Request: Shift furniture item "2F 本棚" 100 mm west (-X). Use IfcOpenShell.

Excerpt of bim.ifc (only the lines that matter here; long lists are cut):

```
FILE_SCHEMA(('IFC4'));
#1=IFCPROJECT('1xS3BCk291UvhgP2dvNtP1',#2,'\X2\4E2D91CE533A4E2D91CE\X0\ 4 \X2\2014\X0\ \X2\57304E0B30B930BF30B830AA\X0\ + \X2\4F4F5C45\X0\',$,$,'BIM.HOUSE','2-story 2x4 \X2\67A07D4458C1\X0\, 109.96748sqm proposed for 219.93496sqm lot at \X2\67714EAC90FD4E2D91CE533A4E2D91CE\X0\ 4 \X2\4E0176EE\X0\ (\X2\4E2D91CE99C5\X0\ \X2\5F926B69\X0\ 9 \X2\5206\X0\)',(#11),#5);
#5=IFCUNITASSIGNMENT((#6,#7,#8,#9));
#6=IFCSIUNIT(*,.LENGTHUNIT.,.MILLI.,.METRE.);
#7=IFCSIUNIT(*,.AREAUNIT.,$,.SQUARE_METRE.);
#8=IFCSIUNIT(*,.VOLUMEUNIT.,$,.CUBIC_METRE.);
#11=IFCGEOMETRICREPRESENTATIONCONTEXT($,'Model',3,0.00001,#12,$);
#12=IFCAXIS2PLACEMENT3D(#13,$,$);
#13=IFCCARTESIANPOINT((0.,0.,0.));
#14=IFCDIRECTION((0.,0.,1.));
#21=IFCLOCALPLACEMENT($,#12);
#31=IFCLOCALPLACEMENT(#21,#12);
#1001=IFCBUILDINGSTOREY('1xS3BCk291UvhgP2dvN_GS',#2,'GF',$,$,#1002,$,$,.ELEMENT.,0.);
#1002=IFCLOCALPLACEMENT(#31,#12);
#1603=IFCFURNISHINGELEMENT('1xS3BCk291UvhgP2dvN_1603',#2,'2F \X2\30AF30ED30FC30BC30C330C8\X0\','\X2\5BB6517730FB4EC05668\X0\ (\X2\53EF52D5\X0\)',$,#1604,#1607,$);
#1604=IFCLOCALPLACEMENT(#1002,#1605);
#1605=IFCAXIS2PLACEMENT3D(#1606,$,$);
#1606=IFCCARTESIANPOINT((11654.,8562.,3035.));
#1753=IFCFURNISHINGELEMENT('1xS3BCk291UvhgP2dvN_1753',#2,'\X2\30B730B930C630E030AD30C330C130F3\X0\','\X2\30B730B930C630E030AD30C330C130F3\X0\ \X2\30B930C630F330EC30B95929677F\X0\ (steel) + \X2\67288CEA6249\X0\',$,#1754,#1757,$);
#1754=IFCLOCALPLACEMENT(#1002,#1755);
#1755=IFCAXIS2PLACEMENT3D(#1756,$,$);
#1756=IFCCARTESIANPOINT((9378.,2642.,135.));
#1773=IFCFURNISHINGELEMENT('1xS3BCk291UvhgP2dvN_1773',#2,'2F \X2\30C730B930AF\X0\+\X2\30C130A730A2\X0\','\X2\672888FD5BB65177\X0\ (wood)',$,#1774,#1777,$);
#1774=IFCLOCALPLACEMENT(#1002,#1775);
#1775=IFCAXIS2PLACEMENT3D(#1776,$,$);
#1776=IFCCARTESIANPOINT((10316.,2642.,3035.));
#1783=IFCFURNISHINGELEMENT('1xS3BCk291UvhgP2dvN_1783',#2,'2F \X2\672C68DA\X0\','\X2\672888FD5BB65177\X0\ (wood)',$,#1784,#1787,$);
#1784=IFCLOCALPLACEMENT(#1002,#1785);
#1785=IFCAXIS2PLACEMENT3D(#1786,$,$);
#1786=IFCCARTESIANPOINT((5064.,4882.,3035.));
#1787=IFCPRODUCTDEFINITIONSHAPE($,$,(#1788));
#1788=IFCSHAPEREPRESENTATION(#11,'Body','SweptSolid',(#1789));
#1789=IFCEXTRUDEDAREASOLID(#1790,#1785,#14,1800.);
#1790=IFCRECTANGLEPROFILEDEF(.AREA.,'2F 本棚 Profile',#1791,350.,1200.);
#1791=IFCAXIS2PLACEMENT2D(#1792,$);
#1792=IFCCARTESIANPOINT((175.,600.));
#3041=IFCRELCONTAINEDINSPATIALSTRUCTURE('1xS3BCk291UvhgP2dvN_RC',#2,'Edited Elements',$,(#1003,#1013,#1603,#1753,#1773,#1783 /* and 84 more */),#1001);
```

```python
import ifcopenshell
import ifcopenshell.api.geometry
import ifcopenshell.util.placement
import ifcopenshell.util.unit

model = ifcopenshell.open("bim.ifc")
unit_scale = ifcopenshell.util.unit.calculate_unit_scale(model)

item = model.by_guid("1xS3BCk291UvhgP2dvN_1783")
matrix = ifcopenshell.util.placement.get_local_placement(item.ObjectPlacement)
matrix[0, 3] -= 0.1 / unit_scale
ifcopenshell.api.geometry.edit_object_placement(model, product=item, matrix=matrix, is_si=False)

print(ifcopenshell.util.placement.get_local_placement(item.ObjectPlacement).round(3) + 0.0)

model.write("bim_v2.ifc")
```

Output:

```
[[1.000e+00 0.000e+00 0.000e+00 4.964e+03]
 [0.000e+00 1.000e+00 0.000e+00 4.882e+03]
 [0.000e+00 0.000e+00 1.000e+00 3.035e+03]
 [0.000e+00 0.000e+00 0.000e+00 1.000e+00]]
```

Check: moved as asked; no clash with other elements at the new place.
